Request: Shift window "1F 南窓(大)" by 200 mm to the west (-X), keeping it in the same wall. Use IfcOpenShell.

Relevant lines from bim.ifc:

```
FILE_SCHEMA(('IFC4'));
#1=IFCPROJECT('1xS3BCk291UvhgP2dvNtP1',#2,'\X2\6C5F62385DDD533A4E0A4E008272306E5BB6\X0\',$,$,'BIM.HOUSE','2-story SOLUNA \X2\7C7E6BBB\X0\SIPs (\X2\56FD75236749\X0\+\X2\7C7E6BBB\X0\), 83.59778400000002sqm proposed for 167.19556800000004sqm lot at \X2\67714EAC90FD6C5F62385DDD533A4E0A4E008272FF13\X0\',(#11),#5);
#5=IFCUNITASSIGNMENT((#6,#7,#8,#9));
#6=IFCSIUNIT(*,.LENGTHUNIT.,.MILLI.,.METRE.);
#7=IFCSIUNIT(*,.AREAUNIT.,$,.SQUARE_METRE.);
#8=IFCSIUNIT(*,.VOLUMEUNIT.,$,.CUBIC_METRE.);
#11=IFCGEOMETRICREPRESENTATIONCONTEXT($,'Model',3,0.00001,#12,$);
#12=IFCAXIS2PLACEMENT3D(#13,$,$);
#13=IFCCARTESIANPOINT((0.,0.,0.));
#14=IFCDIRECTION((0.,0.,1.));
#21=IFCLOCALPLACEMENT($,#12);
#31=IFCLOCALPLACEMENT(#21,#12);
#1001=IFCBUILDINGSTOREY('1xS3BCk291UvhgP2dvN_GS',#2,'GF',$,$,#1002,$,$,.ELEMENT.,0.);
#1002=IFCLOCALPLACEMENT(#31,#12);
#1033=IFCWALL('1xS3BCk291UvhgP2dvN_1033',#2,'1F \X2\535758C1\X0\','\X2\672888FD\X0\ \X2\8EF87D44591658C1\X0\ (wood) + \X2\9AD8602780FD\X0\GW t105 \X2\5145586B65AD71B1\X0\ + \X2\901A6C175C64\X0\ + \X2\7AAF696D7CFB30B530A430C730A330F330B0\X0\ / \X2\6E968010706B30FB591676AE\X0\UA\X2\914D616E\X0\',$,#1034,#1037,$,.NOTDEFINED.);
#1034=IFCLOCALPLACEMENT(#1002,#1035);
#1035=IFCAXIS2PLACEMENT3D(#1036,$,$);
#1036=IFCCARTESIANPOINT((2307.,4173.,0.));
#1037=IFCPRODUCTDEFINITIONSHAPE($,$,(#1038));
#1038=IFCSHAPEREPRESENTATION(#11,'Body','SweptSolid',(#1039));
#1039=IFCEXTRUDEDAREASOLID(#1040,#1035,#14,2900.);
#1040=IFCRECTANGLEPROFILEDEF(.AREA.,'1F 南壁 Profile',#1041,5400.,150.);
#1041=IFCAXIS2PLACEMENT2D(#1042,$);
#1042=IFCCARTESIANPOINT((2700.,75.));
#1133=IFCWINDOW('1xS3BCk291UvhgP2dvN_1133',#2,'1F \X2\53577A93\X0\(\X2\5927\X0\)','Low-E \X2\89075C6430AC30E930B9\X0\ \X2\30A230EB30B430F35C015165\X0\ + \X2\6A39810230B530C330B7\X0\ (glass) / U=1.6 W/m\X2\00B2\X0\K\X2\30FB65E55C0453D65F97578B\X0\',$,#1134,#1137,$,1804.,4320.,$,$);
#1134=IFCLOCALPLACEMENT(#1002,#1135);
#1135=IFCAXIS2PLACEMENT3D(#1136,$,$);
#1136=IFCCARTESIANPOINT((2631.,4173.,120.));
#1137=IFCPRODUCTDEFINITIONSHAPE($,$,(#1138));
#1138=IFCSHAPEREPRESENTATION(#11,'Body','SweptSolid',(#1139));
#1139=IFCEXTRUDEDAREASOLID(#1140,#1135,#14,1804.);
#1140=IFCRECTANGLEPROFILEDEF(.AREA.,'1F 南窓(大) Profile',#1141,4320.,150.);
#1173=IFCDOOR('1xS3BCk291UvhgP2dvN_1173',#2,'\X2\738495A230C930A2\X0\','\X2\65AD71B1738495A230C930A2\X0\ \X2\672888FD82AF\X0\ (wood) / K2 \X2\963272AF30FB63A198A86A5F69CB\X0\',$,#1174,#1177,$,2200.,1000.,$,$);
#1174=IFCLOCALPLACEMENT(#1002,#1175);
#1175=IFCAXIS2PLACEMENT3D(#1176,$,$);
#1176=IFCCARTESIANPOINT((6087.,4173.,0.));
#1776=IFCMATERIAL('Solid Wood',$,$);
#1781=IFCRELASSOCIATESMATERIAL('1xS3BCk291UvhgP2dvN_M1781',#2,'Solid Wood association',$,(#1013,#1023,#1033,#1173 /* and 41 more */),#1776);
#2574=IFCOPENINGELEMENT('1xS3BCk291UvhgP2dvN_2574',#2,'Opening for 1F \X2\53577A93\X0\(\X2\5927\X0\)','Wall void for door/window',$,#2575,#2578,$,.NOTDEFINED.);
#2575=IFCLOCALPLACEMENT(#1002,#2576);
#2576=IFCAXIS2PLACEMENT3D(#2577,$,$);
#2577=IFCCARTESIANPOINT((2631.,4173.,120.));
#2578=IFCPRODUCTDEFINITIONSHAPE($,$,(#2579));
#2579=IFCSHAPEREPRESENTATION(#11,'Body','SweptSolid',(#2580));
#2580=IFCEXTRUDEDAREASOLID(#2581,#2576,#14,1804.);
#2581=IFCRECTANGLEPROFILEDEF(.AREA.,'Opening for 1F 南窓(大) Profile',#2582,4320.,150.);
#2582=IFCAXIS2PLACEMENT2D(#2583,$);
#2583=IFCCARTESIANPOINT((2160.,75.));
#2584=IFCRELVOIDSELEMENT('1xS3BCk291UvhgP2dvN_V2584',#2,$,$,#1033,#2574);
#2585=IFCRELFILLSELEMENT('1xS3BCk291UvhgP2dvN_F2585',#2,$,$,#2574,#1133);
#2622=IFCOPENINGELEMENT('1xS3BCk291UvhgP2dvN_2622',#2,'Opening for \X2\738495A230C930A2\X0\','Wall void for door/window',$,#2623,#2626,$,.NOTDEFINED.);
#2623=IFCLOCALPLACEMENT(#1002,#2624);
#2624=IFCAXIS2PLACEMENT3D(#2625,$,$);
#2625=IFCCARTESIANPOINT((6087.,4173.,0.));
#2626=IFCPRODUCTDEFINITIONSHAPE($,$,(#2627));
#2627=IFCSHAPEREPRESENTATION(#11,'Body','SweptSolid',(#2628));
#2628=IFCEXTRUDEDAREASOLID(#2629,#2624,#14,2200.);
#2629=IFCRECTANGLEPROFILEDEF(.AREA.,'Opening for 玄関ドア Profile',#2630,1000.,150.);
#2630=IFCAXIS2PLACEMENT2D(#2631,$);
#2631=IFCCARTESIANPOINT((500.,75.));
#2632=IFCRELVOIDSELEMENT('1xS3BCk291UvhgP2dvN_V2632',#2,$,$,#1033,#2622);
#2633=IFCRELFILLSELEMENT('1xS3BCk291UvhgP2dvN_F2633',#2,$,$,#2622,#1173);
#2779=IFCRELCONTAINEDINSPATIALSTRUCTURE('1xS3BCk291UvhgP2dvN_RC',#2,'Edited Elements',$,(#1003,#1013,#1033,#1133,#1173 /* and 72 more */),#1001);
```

```python
import ifcopenshell
import ifcopenshell.api.geometry
import ifcopenshell.util.placement

model = ifcopenshell.open("bim.ifc")

window = model.by_id(1133)
opening = window.FillsVoids[0].RelatingOpeningElement
wall = opening.VoidsElements[0].RelatingBuildingElement

wall_matrix = ifcopenshell.util.placement.get_local_placement(wall.ObjectPlacement)
shift = wall_matrix[:3, 0] * -200.0
before = ifcopenshell.util.placement.get_local_placement(window.ObjectPlacement)[:3, 3].copy()

# The window is not placed relative to its opening, so move both.
for product in (opening, window):
    matrix = ifcopenshell.util.placement.get_local_placement(product.ObjectPlacement)
    matrix[:3, 3] += shift
    ifcopenshell.api.geometry.edit_object_placement(model, product=product, matrix=matrix, is_si=False)

after = ifcopenshell.util.placement.get_local_placement(window.ObjectPlacement)[:3, 3]
print("window moved by", (after - before).round(3) + 0.0)

model.write("bim_rev.ifc")
```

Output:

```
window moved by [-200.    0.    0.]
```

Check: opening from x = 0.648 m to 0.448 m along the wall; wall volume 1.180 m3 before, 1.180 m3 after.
